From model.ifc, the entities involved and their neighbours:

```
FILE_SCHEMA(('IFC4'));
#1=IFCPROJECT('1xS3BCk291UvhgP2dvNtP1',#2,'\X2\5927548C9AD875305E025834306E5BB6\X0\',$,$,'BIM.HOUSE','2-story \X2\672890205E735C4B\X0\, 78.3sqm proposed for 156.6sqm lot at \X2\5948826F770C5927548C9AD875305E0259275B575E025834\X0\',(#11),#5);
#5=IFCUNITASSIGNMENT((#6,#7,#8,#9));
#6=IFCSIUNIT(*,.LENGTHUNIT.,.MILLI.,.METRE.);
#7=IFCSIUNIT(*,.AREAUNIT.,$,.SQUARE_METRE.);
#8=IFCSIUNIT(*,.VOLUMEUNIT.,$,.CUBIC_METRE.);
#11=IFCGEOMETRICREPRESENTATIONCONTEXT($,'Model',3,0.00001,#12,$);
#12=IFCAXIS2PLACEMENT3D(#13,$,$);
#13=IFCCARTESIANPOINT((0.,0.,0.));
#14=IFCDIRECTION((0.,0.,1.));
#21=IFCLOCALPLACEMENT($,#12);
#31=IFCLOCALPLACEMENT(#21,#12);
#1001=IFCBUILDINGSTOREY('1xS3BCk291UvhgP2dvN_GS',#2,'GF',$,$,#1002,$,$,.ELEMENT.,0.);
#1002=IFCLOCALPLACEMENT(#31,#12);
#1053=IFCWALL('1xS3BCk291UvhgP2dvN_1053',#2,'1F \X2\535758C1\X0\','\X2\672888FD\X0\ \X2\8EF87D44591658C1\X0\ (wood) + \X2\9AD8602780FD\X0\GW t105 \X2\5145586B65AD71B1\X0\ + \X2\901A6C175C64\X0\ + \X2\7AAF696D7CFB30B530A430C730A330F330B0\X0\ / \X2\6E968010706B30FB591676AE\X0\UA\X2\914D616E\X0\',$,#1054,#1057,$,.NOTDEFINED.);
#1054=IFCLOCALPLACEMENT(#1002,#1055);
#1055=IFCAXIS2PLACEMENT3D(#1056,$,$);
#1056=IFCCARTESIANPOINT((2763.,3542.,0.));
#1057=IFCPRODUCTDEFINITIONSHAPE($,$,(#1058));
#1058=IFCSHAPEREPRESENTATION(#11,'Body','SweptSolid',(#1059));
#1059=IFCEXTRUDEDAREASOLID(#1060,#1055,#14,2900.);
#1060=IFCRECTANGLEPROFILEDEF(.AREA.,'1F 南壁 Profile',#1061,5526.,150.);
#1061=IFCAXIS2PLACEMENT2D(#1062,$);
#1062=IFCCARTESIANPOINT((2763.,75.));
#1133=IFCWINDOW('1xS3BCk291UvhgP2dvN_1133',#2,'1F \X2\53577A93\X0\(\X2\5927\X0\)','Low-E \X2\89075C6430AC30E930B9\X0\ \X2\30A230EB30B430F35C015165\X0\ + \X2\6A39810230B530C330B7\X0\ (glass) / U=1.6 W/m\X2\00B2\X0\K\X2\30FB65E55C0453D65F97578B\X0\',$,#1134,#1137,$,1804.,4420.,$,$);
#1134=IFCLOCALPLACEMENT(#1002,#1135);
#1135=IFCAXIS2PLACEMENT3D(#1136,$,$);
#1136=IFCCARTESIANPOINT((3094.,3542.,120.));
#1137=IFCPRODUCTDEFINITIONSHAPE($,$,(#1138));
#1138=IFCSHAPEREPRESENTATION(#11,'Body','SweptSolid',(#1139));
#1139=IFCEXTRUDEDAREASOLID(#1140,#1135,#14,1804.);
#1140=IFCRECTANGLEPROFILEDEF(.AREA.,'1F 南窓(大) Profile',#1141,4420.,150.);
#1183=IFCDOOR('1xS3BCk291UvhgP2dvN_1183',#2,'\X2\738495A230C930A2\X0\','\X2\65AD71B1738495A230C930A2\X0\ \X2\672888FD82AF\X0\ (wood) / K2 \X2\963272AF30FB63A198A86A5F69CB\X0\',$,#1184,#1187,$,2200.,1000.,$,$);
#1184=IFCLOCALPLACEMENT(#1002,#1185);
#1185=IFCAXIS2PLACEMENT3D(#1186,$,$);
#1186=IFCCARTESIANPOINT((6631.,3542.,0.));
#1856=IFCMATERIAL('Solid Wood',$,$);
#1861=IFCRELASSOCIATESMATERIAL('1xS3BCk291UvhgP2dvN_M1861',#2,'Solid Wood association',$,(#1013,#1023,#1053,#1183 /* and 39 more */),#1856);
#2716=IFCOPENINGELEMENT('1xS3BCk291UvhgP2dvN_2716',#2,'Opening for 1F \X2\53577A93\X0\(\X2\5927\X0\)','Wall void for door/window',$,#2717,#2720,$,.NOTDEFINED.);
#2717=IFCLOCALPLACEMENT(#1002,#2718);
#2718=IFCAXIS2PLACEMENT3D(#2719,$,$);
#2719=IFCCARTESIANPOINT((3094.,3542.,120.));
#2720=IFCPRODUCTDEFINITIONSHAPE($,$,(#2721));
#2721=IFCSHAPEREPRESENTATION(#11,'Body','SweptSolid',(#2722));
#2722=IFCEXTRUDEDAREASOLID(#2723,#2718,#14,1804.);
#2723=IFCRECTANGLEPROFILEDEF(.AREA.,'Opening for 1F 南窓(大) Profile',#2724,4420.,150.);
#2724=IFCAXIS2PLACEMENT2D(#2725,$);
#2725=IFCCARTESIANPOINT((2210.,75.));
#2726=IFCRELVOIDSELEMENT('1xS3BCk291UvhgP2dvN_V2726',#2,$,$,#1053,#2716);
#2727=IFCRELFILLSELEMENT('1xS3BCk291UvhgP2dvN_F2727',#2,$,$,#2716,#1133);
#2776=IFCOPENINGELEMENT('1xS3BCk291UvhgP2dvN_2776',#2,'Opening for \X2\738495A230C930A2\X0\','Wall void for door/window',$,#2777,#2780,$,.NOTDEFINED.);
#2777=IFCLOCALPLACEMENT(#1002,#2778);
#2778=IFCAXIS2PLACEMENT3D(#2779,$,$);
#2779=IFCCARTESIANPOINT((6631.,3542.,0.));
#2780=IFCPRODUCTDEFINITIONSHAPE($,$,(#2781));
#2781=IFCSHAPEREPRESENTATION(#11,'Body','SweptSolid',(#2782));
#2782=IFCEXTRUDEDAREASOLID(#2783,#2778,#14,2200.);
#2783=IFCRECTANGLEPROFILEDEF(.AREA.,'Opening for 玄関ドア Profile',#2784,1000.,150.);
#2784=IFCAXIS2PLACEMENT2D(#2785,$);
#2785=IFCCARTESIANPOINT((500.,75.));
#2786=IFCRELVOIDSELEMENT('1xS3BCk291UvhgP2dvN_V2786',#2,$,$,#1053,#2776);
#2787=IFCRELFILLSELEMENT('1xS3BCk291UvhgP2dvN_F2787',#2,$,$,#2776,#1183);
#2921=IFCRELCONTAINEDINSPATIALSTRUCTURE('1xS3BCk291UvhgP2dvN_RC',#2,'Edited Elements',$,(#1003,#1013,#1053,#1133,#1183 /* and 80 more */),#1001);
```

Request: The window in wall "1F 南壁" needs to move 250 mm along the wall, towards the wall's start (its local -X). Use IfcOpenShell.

```python
import ifcopenshell
import ifcopenshell.api.geometry
import ifcopenshell.util.placement
import ifcopenshell.util.unit

model = ifcopenshell.open("model.ifc")
unit_scale = ifcopenshell.util.unit.calculate_unit_scale(model)

window = model.by_guid("1xS3BCk291UvhgP2dvN_1133")
opening = window.FillsVoids[0].RelatingOpeningElement
wall = opening.VoidsElements[0].RelatingBuildingElement

wall_matrix = ifcopenshell.util.placement.get_local_placement(wall.ObjectPlacement)
shift = wall_matrix[:3, 0] * -0.25 / unit_scale
before = ifcopenshell.util.placement.get_local_placement(window.ObjectPlacement)[:3, 3].copy()

# The window is not placed relative to its opening, so move both.
for product in (opening, window):
    matrix = ifcopenshell.util.placement.get_local_placement(product.ObjectPlacement)
    matrix[:3, 3] += shift
    ifcopenshell.api.geometry.edit_object_placement(model, product=product, matrix=matrix, is_si=False)

after = ifcopenshell.util.placement.get_local_placement(window.ObjectPlacement)[:3, 3]
print("window moved by", (after - before).round(3) + 0.0)

model.write("model_updated.ifc")
```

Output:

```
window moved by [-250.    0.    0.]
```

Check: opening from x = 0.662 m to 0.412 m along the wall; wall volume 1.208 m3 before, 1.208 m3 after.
